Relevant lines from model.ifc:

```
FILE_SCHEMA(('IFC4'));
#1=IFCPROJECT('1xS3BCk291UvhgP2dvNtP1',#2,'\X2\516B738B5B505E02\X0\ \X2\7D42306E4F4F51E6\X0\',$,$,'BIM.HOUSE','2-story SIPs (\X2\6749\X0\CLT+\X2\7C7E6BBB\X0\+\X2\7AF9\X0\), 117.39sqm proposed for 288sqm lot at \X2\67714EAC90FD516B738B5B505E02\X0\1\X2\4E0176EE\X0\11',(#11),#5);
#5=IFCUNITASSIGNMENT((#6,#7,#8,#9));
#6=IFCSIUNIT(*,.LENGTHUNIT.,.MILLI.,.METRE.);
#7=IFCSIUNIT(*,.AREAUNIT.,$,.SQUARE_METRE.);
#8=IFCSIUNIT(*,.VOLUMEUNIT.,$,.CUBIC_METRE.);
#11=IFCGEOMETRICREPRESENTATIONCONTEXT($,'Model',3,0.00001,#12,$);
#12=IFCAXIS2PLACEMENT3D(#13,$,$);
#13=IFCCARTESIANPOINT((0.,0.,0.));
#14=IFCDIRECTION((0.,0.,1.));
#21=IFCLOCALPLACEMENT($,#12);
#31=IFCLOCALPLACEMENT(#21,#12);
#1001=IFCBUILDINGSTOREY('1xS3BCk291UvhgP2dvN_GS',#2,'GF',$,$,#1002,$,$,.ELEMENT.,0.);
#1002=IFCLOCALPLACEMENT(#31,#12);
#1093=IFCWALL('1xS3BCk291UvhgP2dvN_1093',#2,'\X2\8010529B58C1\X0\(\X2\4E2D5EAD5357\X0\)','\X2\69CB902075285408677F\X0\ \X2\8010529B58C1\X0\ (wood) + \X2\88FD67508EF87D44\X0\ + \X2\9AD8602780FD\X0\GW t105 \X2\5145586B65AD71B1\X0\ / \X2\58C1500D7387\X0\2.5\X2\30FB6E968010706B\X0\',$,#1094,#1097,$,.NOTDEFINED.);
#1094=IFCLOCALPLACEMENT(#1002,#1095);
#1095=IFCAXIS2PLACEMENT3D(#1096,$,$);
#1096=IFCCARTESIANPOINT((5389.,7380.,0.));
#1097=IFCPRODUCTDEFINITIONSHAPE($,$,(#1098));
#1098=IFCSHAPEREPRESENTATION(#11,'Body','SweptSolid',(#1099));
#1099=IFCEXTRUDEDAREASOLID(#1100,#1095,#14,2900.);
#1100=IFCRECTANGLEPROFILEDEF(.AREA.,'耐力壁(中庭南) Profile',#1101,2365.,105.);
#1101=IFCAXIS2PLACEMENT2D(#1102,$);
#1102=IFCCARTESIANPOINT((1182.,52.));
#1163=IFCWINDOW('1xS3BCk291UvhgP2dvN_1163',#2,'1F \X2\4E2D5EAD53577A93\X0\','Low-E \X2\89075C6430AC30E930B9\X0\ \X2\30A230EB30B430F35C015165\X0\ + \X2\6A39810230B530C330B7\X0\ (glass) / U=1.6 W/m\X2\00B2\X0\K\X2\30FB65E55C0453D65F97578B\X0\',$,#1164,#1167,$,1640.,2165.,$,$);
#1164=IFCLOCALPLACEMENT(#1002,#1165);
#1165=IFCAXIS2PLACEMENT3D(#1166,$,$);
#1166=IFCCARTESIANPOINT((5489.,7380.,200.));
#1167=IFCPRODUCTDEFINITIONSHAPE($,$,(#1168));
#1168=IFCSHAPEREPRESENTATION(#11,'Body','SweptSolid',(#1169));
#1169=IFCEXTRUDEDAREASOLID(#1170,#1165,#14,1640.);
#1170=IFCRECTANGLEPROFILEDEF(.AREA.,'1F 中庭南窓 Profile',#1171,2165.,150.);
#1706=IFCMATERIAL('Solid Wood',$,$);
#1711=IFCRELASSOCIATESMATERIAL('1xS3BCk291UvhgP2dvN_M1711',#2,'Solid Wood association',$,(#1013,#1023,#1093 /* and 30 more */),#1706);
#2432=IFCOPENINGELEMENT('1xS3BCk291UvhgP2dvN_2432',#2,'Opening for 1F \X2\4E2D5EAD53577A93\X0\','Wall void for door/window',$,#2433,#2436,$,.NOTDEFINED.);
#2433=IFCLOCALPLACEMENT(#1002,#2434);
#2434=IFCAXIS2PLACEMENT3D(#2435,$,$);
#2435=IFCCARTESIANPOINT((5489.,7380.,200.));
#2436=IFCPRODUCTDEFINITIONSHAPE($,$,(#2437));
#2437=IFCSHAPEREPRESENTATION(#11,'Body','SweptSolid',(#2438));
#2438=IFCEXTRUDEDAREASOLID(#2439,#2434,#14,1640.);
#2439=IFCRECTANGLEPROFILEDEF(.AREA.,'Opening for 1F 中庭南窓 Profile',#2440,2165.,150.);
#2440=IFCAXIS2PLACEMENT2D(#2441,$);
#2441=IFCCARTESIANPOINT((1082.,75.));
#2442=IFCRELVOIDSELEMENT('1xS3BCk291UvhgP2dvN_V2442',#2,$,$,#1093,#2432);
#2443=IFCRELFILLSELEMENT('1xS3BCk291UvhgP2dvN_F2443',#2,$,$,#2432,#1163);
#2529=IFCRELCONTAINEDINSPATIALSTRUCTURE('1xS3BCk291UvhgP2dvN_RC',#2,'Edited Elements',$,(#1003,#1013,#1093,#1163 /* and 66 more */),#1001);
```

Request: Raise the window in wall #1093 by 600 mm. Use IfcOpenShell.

```python
import numpy as np
import ifcopenshell
import ifcopenshell.api.geometry
import ifcopenshell.util.placement
import ifcopenshell.util.unit

model = ifcopenshell.open("model.ifc")
unit_scale = ifcopenshell.util.unit.calculate_unit_scale(model)

window = model.by_guid("1xS3BCk291UvhgP2dvN_1163")
opening = window.FillsVoids[0].RelatingOpeningElement
dz = 0.6 / unit_scale

shift = np.array([0.0, 0.0, dz])
# The window is not placed relative to its opening, so move both.
for product in (opening, window):
    matrix = ifcopenshell.util.placement.get_local_placement(product.ObjectPlacement)
    matrix[:3, 3] += shift
    ifcopenshell.api.geometry.edit_object_placement(model, product=product, matrix=matrix, is_si=False)

print(f"moved by {dz * unit_scale:+.3f} m")

model.write("model_v2.ifc")
```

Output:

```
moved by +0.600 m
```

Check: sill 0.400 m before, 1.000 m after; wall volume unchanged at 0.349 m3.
